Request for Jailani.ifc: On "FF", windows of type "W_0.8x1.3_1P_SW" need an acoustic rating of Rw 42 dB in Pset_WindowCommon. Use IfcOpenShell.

First a look at what the model holds.

```python
import ifcopenshell
import ifcopenshell.util.element

model = ifcopenshell.open("Jailani.ifc")
print(model.schema)
storey = next(s for s in model.by_type("IfcBuildingStorey") if s.Name == "FF")
windows = [e for e in ifcopenshell.util.element.get_decomposition(storey) if e.is_a("IfcWindow")]
seen = {}
for e in windows:
    element_type = ifcopenshell.util.element.get_type(e)
    key = (element_type.Name if element_type != e and element_type else None, ifcopenshell.util.element.get_pset(e, "Pset_WindowCommon", "AcousticRating"))
    seen[key] = seen.get(key, 0) + 1
for (name, value), count in sorted(seen.items(), key=str):
    print(count, "x", name, "|", value)
```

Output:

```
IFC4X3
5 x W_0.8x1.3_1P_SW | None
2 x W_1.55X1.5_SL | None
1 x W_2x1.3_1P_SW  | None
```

```python
import ifcopenshell
import ifcopenshell.api.pset
import ifcopenshell.util.element

model = ifcopenshell.open("Jailani.ifc")

storey = next(s for s in model.by_type("IfcBuildingStorey") if s.Name == "FF")
windows = [e for e in ifcopenshell.util.element.get_decomposition(storey) if e.is_a("IfcWindow")]

count = 0
for e in windows:
    element_type = ifcopenshell.util.element.get_type(e)
    if element_type in (None, e) or element_type.Name != "W_0.8x1.3_1P_SW":
        continue
    # add_pset returns the element's existing set when there is one.
    pset = ifcopenshell.api.pset.add_pset(model, product=e, name="Pset_WindowCommon")
    ifcopenshell.api.pset.edit_pset(model, pset=pset, properties={"AcousticRating": "Rw 42 dB"})
    count += 1

print(count, "windows updated")

model.write("Jailani_v2.ifc")
```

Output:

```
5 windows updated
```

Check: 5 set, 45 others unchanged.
